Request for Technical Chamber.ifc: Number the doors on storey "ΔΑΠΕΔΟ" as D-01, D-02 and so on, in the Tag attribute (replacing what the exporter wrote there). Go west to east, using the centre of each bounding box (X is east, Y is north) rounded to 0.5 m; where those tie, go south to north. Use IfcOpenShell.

First a look at what the model holds.

```python
import ifcopenshell
import ifcopenshell.util.element
import ifcopenshell.util.placement

model = ifcopenshell.open("Technical Chamber.ifc")
print(model.schema)
storey = next(s for s in model.by_type("IfcBuildingStorey") if s.Name == "ΔΑΠΕΔΟ")
doors = [e for e in ifcopenshell.util.element.get_decomposition(storey) if e.is_a("IfcDoor")]
for e in sorted(doors, key=lambda e: e.id()):
    origin = ifcopenshell.util.placement.get_local_placement(e.ObjectPlacement)[:3, 3]
    print(e.id(), e.Tag, e.Name, origin.round(2) + 0.0, sep=" | ")
```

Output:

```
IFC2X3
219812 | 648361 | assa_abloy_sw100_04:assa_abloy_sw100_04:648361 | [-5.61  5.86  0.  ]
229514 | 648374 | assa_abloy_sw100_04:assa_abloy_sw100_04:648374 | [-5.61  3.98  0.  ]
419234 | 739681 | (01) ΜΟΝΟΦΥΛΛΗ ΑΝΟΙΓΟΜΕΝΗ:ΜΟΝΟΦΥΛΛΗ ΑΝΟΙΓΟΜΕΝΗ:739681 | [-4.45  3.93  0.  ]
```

```python
import ifcopenshell
import ifcopenshell.geom
import ifcopenshell.util.element
import ifcopenshell.util.shape

model = ifcopenshell.open("Technical Chamber.ifc")
settings = ifcopenshell.geom.settings()
settings.set("use-world-coords", True)


def centre(element):
    shape = ifcopenshell.geom.create_shape(settings, element)
    return ifcopenshell.util.shape.get_bbox_centroid(shape.geometry)


storey = next(s for s in model.by_type("IfcBuildingStorey") if s.Name == "ΔΑΠΕΔΟ")
doors = [e for e in ifcopenshell.util.element.get_decomposition(storey) if e.is_a("IfcDoor")]

# Insertion points can sit at a corner or the storey origin, so sort by the geometry (in metres).
centres = {e: centre(e) for e in doors}
doors.sort(key=lambda e: (round(centres[e][0] / 0.5), centres[e][1]))

for i, e in enumerate(doors, start=1):
    number = f"D-{i:02d}"
    e.Tag = number
    print(e.id(), number)

model.write("Technical Chamber_v2.ifc")
```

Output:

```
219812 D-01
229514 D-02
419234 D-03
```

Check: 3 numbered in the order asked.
